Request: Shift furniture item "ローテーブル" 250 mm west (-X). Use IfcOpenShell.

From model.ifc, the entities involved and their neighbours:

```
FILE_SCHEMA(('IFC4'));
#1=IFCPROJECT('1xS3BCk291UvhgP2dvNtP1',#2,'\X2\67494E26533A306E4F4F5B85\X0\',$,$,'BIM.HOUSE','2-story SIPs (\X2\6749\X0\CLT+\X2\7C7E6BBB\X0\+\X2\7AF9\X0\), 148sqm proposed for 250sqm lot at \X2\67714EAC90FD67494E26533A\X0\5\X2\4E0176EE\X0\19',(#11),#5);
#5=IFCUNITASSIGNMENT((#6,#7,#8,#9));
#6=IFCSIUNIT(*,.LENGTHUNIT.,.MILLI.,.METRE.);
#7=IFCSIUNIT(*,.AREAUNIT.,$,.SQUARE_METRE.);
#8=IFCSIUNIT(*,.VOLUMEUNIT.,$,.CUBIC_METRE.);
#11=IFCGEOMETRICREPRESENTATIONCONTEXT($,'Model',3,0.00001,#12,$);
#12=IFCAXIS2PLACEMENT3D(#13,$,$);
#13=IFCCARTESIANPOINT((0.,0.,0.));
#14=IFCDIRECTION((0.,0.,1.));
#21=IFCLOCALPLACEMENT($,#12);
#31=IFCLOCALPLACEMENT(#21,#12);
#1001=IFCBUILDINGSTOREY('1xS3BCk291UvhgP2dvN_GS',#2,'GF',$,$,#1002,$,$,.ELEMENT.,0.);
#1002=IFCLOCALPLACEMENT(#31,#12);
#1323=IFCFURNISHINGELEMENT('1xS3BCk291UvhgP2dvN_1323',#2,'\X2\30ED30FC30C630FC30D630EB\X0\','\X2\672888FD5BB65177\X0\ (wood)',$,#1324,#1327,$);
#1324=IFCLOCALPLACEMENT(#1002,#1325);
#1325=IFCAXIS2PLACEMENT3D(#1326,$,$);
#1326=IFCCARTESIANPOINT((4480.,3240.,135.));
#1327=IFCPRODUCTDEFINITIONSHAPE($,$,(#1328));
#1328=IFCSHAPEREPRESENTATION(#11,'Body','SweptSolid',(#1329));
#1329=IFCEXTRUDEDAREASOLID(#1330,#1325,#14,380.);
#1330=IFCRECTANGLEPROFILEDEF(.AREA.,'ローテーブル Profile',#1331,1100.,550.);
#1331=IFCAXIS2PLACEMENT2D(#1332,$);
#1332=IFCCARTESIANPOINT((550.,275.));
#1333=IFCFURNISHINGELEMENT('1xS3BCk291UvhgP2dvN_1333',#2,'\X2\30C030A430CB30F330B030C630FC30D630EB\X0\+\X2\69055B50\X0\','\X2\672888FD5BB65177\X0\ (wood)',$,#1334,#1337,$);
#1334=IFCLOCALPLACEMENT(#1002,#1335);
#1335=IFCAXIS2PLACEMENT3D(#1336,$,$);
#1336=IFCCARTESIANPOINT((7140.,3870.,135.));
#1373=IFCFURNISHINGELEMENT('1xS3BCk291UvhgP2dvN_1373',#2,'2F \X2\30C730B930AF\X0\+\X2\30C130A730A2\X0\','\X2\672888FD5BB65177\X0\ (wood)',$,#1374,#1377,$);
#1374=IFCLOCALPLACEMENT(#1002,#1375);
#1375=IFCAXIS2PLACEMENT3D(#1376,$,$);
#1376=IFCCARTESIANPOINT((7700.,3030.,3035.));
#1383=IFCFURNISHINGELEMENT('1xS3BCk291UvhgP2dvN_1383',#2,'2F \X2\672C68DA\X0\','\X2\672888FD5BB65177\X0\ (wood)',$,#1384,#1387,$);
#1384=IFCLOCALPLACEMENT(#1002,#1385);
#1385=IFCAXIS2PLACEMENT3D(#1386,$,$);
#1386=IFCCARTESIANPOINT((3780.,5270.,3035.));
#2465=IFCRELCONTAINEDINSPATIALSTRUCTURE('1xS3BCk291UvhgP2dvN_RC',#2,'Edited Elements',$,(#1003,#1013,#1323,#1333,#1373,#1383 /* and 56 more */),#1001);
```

```python
import ifcopenshell
import ifcopenshell.api.geometry
import ifcopenshell.util.placement

model = ifcopenshell.open("model.ifc")

item = model.by_guid("1xS3BCk291UvhgP2dvN_1323")
matrix = ifcopenshell.util.placement.get_local_placement(item.ObjectPlacement)
matrix[0, 3] -= 250.0
ifcopenshell.api.geometry.edit_object_placement(model, product=item, matrix=matrix, is_si=False)

print(ifcopenshell.util.placement.get_local_placement(item.ObjectPlacement).round(3) + 0.0)

model.write("model_updated.ifc")
```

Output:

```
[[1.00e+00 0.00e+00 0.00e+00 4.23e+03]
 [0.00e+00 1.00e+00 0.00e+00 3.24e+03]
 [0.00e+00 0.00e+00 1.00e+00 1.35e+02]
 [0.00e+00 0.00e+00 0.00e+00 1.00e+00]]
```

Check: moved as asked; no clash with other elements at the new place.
